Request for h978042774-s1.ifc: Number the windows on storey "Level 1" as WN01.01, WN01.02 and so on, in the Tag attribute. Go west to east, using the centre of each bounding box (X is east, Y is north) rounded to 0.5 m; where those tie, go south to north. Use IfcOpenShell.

First a look at what the model holds.

```python
import ifcopenshell
import ifcopenshell.util.element
import ifcopenshell.util.placement

model = ifcopenshell.open("h978042774-s1.ifc")
print(model.schema)
storey = next(s for s in model.by_type("IfcBuildingStorey") if s.Name == "Level 1")
windows = [e for e in ifcopenshell.util.element.get_decomposition(storey) if e.is_a("IfcWindow")]
for e in sorted(windows, key=lambda e: e.id()):
    origin = ifcopenshell.util.placement.get_local_placement(e.ObjectPlacement)[:3, 3]
    print(e.id(), e.Tag, e.Name, origin.round(2) + 0.0, sep=" | ")
```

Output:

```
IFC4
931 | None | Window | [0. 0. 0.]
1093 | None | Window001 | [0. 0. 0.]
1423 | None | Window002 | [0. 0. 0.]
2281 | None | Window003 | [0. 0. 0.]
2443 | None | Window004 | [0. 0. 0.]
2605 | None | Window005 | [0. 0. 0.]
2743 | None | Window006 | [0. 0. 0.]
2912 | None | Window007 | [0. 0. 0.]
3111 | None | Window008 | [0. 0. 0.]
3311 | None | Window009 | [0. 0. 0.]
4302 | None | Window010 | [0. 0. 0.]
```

```python
import ifcopenshell
import ifcopenshell.geom
import ifcopenshell.util.element
import ifcopenshell.util.shape

model = ifcopenshell.open("h978042774-s1.ifc")
settings = ifcopenshell.geom.settings()
settings.set("use-world-coords", True)


def centre(element):
    shape = ifcopenshell.geom.create_shape(settings, element)
    return ifcopenshell.util.shape.get_bbox_centroid(shape.geometry)


storey = next(s for s in model.by_type("IfcBuildingStorey") if s.Name == "Level 1")
windows = [e for e in ifcopenshell.util.element.get_decomposition(storey) if e.is_a("IfcWindow")]

# Insertion points can sit at a corner or the storey origin, so sort by the geometry (in metres).
centres = {e: centre(e) for e in windows}
windows.sort(key=lambda e: (round(centres[e][0] / 0.5), centres[e][1]))

for i, e in enumerate(windows, start=1):
    number = f"WN01.{i:02d}"
    e.Tag = number
    print(e.id(), number)

model.write("h978042774-s1_updated.ifc")
```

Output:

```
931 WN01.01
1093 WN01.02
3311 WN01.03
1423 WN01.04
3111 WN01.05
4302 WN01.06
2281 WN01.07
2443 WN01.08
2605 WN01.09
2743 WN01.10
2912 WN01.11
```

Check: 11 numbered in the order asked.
